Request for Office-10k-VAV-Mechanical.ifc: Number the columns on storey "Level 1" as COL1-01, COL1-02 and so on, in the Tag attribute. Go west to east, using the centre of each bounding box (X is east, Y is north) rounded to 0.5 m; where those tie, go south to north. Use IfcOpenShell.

First a look at what the model holds.

```python
import ifcopenshell
import ifcopenshell.util.element
import ifcopenshell.util.placement

model = ifcopenshell.open("Office-10k-VAV-Mechanical.ifc")
print(model.schema)
storey = next(s for s in model.by_type("IfcBuildingStorey") if s.Name == "Level 1")
columns = [e for e in ifcopenshell.util.element.get_decomposition(storey) if e.is_a("IfcColumn")]
for e in sorted(columns, key=lambda e: e.id()):
    origin = ifcopenshell.util.placement.get_local_placement(e.ObjectPlacement)[:3, 3]
    print(e.id(), e.Tag, e.Name, origin.round(2) + 0.0, sep=" | ")
```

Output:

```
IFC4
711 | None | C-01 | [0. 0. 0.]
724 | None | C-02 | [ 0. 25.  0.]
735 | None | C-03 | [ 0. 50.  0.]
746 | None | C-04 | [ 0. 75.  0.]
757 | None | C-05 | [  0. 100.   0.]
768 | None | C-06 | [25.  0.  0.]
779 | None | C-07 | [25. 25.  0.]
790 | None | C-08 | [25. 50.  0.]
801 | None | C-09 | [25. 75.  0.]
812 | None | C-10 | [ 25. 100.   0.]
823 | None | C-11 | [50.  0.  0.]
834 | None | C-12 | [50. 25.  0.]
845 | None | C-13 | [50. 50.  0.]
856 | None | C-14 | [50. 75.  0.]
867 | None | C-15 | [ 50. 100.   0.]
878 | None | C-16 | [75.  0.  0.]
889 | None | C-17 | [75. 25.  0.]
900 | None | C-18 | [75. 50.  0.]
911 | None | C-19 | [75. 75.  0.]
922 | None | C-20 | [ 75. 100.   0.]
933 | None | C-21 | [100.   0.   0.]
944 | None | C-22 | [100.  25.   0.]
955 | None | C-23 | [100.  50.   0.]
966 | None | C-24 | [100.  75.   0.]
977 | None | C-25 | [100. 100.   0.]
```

```python
import ifcopenshell
import ifcopenshell.geom
import ifcopenshell.util.element
import ifcopenshell.util.shape

model = ifcopenshell.open("Office-10k-VAV-Mechanical.ifc")
settings = ifcopenshell.geom.settings()
settings.set("use-world-coords", True)


def centre(element):
    shape = ifcopenshell.geom.create_shape(settings, element)
    return ifcopenshell.util.shape.get_bbox_centroid(shape.geometry)


storey = next(s for s in model.by_type("IfcBuildingStorey") if s.Name == "Level 1")
columns = [e for e in ifcopenshell.util.element.get_decomposition(storey) if e.is_a("IfcColumn")]

# Insertion points can sit at a corner or the storey origin, so sort by the geometry (in metres).
centres = {e: centre(e) for e in columns}
columns.sort(key=lambda e: (round(centres[e][0] / 0.5), centres[e][1]))

for i, e in enumerate(columns, start=1):
    number = f"COL1-{i:02d}"
    e.Tag = number
    print(e.id(), number)

model.write("Office-10k-VAV-Mechanical_rev.ifc")
```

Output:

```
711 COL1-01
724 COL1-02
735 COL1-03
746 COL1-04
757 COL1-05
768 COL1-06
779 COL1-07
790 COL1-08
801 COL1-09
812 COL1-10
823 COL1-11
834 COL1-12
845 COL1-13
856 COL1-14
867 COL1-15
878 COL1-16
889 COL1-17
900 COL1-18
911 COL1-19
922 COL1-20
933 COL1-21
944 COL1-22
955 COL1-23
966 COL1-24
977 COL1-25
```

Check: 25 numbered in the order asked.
